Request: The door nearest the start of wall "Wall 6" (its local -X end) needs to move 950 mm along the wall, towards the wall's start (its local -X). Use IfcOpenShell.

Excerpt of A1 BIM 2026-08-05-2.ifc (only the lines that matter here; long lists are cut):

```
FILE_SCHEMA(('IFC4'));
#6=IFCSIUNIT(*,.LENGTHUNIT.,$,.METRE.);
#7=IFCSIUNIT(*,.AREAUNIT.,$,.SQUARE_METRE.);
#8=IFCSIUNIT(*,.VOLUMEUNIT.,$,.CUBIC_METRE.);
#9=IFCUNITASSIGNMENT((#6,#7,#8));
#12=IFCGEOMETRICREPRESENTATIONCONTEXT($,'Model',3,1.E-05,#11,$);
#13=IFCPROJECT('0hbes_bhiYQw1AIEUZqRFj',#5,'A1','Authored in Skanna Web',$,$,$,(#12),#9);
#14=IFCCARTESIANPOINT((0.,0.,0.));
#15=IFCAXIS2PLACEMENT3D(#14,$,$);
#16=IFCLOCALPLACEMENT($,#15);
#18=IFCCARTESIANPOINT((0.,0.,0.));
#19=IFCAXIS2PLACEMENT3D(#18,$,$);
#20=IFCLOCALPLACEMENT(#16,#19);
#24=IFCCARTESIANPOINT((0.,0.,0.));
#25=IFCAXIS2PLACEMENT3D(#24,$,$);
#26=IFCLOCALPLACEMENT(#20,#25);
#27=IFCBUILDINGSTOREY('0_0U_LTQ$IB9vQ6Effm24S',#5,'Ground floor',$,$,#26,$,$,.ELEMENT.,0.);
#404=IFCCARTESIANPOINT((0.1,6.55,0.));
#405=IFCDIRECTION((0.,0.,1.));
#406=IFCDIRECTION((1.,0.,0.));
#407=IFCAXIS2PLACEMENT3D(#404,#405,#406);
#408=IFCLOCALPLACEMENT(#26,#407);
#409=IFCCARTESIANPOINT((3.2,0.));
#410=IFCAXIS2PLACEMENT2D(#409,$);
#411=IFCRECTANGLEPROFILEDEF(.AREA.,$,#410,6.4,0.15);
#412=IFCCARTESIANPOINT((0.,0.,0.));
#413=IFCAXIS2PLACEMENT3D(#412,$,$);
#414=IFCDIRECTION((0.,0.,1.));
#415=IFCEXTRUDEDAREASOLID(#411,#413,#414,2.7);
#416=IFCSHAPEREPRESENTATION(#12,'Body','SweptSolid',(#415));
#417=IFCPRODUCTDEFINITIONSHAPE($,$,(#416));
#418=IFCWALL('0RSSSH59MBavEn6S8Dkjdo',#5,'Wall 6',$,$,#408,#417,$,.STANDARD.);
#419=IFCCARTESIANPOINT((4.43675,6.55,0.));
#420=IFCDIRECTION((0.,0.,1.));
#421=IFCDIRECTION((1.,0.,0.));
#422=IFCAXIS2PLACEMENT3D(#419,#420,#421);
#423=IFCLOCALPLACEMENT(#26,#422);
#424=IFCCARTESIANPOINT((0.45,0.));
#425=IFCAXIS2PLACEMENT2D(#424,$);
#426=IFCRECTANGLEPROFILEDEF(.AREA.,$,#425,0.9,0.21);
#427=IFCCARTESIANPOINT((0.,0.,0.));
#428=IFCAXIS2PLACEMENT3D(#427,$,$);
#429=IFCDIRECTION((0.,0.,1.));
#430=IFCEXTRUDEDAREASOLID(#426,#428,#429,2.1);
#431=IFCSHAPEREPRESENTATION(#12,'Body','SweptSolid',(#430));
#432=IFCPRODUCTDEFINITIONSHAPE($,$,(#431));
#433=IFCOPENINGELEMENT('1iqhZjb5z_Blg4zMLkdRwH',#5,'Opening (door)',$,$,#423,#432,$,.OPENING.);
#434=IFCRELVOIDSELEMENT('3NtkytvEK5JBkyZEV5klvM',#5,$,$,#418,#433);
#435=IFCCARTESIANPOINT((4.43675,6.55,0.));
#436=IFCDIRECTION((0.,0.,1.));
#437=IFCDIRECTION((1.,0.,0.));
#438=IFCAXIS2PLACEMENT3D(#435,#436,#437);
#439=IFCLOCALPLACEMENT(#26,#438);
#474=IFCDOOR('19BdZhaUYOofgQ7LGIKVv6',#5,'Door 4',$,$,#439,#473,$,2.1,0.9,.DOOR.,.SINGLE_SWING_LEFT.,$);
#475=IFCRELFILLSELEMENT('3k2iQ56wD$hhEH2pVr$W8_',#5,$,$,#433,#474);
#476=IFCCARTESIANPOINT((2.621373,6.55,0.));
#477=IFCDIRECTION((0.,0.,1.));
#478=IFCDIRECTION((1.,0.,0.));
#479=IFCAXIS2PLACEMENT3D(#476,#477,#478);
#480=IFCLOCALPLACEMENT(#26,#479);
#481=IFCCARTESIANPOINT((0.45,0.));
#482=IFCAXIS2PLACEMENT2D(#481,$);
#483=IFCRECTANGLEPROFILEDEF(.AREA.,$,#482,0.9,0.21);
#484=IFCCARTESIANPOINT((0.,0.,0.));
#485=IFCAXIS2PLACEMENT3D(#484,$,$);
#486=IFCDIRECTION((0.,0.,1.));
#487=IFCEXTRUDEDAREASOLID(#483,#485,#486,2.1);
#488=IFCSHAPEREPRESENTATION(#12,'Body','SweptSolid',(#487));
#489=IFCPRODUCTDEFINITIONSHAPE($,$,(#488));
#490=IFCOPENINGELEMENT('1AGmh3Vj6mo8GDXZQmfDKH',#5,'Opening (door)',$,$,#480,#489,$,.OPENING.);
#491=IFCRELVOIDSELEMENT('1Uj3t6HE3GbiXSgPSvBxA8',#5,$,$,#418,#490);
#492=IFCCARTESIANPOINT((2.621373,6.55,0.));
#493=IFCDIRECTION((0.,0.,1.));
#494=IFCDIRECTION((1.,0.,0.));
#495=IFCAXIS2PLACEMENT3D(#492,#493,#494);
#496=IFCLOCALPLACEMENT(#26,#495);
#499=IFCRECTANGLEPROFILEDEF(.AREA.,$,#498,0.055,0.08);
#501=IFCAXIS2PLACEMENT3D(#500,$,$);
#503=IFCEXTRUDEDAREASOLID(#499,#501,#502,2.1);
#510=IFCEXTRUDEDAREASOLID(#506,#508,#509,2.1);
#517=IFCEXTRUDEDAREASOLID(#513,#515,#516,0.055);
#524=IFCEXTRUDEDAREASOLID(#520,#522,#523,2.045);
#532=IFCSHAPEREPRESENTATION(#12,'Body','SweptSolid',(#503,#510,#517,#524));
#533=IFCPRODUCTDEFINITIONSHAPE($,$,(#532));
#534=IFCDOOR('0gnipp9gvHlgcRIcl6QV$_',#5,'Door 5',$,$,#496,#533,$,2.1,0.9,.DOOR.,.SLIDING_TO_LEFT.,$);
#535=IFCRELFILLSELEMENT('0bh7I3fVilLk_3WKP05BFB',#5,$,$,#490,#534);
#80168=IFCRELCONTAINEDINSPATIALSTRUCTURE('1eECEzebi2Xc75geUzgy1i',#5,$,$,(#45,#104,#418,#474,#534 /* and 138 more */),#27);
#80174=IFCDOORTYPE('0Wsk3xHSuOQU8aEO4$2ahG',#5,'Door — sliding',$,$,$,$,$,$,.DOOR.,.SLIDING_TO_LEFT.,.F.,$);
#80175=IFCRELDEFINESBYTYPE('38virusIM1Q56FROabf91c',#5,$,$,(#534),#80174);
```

```python
import ifcopenshell
import ifcopenshell.api.geometry
import ifcopenshell.util.placement
import ifcopenshell.util.unit

model = ifcopenshell.open("A1 BIM 2026-08-05-2.ifc")
unit_scale = ifcopenshell.util.unit.calculate_unit_scale(model)

door = model.by_guid("0gnipp9gvHlgcRIcl6QV$_")
opening = door.FillsVoids[0].RelatingOpeningElement
wall = opening.VoidsElements[0].RelatingBuildingElement

wall_matrix = ifcopenshell.util.placement.get_local_placement(wall.ObjectPlacement)
shift = wall_matrix[:3, 0] * -0.95 / unit_scale
before = ifcopenshell.util.placement.get_local_placement(door.ObjectPlacement)[:3, 3].copy()

# The door is not placed relative to its opening, so move both.
for product in (opening, door):
    matrix = ifcopenshell.util.placement.get_local_placement(product.ObjectPlacement)
    matrix[:3, 3] += shift
    ifcopenshell.api.geometry.edit_object_placement(model, product=product, matrix=matrix, is_si=False)

after = ifcopenshell.util.placement.get_local_placement(door.ObjectPlacement)[:3, 3]
print("door moved by", (after - before).round(3) + 0.0)

model.write("A1 BIM 2026-08-05-2-out.ifc")
```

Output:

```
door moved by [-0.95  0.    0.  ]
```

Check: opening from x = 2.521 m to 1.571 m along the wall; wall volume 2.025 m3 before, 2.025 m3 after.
